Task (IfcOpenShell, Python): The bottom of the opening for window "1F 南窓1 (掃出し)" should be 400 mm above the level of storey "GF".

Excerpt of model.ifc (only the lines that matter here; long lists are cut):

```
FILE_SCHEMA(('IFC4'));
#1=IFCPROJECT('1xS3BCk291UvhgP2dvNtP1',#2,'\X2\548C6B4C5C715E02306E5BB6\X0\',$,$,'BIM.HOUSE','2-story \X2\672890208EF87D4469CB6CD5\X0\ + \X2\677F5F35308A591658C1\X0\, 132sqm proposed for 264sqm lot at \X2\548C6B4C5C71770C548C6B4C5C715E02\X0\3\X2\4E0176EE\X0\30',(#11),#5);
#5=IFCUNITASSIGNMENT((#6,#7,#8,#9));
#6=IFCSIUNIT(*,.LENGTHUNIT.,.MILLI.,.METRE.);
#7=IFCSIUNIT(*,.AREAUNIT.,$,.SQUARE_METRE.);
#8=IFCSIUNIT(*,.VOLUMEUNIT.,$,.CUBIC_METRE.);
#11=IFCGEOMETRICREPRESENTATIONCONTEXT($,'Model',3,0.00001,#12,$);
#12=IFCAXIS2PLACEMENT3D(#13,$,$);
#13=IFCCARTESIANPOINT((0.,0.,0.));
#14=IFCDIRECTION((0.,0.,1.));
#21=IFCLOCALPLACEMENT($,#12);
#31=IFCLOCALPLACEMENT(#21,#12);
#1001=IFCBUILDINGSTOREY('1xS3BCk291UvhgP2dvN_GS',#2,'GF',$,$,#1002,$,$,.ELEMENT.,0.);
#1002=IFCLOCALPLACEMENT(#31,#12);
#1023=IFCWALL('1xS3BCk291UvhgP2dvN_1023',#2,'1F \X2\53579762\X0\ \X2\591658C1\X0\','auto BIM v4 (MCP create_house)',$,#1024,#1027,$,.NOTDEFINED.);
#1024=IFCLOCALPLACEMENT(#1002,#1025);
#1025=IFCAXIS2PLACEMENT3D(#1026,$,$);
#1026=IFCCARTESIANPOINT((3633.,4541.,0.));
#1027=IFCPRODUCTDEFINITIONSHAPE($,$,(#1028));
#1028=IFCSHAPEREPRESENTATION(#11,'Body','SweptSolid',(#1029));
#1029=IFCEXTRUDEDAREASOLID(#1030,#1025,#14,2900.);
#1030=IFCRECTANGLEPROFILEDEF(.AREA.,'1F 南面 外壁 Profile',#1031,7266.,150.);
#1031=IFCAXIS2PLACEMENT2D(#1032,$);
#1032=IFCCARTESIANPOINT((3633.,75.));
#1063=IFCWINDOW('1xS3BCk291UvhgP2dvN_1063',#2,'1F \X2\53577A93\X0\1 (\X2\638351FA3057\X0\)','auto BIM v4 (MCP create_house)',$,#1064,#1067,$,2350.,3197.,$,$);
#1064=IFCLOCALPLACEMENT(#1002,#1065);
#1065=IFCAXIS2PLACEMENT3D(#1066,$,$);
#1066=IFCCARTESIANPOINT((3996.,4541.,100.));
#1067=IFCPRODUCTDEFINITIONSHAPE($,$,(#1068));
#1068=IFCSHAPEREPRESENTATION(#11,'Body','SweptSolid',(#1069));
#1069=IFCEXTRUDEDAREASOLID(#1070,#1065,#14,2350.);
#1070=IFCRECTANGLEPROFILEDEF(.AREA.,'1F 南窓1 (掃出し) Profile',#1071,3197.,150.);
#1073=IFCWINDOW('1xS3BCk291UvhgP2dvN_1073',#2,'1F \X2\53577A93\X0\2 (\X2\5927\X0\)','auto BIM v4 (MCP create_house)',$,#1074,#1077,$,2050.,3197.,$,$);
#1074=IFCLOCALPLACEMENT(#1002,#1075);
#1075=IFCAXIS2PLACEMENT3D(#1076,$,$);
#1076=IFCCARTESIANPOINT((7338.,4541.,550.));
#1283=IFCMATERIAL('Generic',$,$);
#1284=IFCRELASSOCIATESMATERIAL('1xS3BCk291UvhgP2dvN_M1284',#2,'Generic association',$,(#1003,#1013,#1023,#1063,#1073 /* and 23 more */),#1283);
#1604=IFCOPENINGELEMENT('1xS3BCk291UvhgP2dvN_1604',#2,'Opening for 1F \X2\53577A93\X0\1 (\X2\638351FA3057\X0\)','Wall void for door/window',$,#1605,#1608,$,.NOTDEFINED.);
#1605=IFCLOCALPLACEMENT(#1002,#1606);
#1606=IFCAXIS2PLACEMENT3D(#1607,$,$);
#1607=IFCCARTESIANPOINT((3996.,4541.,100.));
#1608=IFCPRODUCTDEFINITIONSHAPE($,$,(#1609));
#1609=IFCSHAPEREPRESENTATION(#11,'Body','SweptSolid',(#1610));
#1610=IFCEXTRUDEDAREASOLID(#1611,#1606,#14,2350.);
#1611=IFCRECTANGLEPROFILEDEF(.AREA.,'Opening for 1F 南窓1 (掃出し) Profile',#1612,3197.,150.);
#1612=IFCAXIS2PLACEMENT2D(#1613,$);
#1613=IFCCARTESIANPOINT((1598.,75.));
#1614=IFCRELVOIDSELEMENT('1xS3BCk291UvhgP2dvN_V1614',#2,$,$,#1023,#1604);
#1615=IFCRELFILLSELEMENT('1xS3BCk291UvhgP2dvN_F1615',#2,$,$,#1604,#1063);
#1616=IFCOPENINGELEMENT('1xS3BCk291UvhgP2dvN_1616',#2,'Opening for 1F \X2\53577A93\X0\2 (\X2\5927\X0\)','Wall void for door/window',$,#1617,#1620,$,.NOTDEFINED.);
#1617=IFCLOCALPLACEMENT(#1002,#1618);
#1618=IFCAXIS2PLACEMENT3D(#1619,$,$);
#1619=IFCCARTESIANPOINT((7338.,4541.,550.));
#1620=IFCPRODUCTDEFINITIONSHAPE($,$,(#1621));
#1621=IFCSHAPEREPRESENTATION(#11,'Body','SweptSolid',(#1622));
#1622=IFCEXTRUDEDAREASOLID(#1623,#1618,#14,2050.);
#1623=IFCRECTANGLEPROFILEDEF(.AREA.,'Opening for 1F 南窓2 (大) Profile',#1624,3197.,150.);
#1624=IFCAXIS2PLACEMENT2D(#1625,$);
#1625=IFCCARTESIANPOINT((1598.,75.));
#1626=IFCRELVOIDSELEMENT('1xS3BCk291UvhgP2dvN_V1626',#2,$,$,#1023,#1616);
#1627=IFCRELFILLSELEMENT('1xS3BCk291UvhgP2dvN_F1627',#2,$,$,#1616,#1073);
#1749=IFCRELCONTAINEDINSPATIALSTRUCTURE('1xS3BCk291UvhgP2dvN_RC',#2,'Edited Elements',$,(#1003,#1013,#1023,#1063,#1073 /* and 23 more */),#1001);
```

```python
import numpy as np
import ifcopenshell
import ifcopenshell.api.geometry
import ifcopenshell.geom
import ifcopenshell.util.element
import ifcopenshell.util.placement
import ifcopenshell.util.shape
import ifcopenshell.util.unit

model = ifcopenshell.open("model.ifc")
unit_scale = ifcopenshell.util.unit.calculate_unit_scale(model)

window = model.by_id(1063)
opening = window.FillsVoids[0].RelatingOpeningElement
storey = ifcopenshell.util.element.get_container(window, ifc_class="IfcBuildingStorey")
level = ifcopenshell.util.placement.get_local_placement(storey.ObjectPlacement)[2, 3]

# The opening's origin need not be at the sill, so measure its lowest point.
shape = ifcopenshell.geom.create_shape(ifcopenshell.geom.settings(), opening)
bottom = ifcopenshell.util.shape.get_shape_bottom_elevation(shape, shape.geometry) / unit_scale
dz = level + 0.4 / unit_scale - bottom

shift = np.array([0.0, 0.0, dz])
# The window is not placed relative to its opening, so move both.
for product in (opening, window):
    matrix = ifcopenshell.util.placement.get_local_placement(product.ObjectPlacement)
    matrix[:3, 3] += shift
    ifcopenshell.api.geometry.edit_object_placement(model, product=product, matrix=matrix, is_si=False)

print(f"moved by {dz * unit_scale:+.3f} m")

model.write("model_updated.ifc")
```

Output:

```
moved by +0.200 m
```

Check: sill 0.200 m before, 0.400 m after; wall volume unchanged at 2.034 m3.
